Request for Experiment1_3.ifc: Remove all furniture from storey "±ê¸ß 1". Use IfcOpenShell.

First a look at what the model holds.

```python
import ifcopenshell
import ifcopenshell.util.element

model = ifcopenshell.open("Experiment1_3.ifc")
print(model.schema)
storey = next(s for s in model.by_type("IfcBuildingStorey") if s.Name == "±ê¸ß 1")
furniture = [e for e in ifcopenshell.util.element.get_decomposition(storey) if e.is_a("IfcFurnishingElement")]
seen = {}
for e in furniture:
    element_type = ifcopenshell.util.element.get_type(e)
    name = element_type.Name if element_type not in (None, e) else None
    seen[name] = seen.get(name, 0) + 1
for name, count in sorted(seen.items(), key=str):
    print(count, "x", name)
```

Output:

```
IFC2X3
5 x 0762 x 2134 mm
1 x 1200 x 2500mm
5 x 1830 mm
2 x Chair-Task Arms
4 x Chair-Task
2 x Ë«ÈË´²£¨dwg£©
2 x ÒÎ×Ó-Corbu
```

```python
import ifcopenshell
import ifcopenshell.api.root
import ifcopenshell.util.element

model = ifcopenshell.open("Experiment1_3.ifc")

storey = next(s for s in model.by_type("IfcBuildingStorey") if s.Name == "±ê¸ß 1")
furniture = [e for e in ifcopenshell.util.element.get_decomposition(storey) if e.is_a("IfcFurnishingElement")]

for e in furniture:
    ifcopenshell.api.root.remove_product(model, product=e)
print(len(furniture), "removed")

model.write("Experiment1_3_rev.ifc")
```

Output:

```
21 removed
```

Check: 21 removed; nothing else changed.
